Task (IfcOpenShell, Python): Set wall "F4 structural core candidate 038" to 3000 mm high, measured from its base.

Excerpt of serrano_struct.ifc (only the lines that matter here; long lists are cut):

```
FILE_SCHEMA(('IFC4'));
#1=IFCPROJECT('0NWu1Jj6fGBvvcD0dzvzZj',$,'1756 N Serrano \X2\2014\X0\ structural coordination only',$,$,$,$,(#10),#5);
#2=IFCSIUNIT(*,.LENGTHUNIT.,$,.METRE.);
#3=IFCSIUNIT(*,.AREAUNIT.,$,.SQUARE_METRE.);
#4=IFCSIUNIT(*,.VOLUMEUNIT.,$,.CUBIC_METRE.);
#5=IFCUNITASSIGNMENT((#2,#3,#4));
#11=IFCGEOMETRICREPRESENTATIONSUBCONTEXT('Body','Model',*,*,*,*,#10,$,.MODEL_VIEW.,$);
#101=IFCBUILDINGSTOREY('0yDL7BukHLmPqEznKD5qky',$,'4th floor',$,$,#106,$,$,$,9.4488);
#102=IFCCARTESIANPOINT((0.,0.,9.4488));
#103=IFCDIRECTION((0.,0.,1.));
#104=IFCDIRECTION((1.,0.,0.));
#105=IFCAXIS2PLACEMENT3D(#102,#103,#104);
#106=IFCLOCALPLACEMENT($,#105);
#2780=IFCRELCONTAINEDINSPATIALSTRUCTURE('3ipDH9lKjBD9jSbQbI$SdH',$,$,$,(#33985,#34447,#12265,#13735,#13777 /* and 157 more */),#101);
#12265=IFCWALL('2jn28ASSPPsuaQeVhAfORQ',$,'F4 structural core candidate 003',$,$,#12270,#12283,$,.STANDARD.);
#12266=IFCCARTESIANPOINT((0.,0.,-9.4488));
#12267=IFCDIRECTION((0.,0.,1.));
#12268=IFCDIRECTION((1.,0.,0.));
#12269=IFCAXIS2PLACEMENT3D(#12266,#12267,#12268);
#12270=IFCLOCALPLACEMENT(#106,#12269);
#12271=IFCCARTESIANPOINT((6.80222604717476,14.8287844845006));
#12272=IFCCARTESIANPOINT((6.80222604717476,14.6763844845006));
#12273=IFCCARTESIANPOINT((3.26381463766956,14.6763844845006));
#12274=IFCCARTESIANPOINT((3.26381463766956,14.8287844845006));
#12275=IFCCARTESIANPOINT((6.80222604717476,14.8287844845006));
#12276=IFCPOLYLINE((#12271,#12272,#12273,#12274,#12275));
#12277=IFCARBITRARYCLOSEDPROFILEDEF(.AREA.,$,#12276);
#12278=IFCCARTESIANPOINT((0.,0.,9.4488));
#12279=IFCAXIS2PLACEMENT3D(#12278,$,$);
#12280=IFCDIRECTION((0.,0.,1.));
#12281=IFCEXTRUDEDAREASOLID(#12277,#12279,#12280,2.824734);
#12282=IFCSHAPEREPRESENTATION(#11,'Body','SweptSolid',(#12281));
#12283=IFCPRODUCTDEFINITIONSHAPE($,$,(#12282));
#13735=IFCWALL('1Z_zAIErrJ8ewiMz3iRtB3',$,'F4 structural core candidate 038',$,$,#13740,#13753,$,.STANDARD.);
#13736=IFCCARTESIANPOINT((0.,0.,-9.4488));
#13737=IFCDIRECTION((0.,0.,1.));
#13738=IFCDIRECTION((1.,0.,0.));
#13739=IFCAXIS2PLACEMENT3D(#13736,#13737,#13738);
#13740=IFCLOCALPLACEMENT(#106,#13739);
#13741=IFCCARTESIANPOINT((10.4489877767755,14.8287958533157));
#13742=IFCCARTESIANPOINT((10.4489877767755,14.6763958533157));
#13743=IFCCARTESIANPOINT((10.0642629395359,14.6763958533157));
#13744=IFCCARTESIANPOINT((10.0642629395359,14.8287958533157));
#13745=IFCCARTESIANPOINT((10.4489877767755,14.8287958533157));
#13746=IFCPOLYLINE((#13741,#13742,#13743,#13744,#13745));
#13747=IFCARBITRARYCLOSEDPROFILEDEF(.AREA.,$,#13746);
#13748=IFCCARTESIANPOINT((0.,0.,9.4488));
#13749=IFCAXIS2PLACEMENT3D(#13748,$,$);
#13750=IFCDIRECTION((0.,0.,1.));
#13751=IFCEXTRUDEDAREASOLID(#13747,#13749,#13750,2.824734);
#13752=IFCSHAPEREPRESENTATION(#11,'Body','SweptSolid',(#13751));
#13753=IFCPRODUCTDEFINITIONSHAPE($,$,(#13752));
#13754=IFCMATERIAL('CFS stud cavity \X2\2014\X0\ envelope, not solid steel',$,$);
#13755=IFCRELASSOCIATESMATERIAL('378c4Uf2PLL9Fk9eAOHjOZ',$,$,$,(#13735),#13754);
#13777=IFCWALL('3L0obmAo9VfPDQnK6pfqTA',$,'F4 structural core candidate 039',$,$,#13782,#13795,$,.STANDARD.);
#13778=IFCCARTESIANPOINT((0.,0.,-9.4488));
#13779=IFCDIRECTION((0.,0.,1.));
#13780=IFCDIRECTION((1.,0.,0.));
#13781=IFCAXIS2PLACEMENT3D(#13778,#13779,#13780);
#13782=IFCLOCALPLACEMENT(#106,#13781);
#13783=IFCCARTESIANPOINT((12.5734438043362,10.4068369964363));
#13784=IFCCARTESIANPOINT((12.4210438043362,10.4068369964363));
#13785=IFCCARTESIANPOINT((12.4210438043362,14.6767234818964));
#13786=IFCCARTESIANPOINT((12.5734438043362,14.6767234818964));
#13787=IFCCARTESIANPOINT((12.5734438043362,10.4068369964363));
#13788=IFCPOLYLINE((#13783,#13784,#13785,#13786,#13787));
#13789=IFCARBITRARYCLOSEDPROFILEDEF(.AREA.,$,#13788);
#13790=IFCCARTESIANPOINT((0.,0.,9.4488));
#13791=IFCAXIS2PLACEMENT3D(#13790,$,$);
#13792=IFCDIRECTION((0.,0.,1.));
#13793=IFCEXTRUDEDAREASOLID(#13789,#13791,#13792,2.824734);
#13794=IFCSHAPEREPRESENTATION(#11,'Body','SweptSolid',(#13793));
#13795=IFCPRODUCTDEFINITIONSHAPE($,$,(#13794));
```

```python
import ifcopenshell
import ifcopenshell.geom
import ifcopenshell.util.representation
import ifcopenshell.util.shape
import ifcopenshell.util.unit

model = ifcopenshell.open("serrano_struct.ifc")
unit_scale = ifcopenshell.util.unit.calculate_unit_scale(model)
settings = ifcopenshell.geom.settings()


def volume(element):
    """Net volume in cubic metres, openings subtracted."""
    shape = ifcopenshell.geom.create_shape(settings, element)
    return ifcopenshell.util.shape.get_volume(shape.geometry)


wall = model.by_guid("1Z_zAIErrJ8ewiMz3iRtB3")
before = volume(wall)

body = ifcopenshell.util.representation.get_representation(wall, "Model", "Body")
solid = body.Items[0]
old_height = solid.Depth
solid.Depth = 3 / unit_scale
after = volume(wall)

print(f"height {old_height:g} -> {solid.Depth:g}, volume {before:.3f} -> {after:.3f} m3")

model.write("serrano_struct_rev.ifc")
```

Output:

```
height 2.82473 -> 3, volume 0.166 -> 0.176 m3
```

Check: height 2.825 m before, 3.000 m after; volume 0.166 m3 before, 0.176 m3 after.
